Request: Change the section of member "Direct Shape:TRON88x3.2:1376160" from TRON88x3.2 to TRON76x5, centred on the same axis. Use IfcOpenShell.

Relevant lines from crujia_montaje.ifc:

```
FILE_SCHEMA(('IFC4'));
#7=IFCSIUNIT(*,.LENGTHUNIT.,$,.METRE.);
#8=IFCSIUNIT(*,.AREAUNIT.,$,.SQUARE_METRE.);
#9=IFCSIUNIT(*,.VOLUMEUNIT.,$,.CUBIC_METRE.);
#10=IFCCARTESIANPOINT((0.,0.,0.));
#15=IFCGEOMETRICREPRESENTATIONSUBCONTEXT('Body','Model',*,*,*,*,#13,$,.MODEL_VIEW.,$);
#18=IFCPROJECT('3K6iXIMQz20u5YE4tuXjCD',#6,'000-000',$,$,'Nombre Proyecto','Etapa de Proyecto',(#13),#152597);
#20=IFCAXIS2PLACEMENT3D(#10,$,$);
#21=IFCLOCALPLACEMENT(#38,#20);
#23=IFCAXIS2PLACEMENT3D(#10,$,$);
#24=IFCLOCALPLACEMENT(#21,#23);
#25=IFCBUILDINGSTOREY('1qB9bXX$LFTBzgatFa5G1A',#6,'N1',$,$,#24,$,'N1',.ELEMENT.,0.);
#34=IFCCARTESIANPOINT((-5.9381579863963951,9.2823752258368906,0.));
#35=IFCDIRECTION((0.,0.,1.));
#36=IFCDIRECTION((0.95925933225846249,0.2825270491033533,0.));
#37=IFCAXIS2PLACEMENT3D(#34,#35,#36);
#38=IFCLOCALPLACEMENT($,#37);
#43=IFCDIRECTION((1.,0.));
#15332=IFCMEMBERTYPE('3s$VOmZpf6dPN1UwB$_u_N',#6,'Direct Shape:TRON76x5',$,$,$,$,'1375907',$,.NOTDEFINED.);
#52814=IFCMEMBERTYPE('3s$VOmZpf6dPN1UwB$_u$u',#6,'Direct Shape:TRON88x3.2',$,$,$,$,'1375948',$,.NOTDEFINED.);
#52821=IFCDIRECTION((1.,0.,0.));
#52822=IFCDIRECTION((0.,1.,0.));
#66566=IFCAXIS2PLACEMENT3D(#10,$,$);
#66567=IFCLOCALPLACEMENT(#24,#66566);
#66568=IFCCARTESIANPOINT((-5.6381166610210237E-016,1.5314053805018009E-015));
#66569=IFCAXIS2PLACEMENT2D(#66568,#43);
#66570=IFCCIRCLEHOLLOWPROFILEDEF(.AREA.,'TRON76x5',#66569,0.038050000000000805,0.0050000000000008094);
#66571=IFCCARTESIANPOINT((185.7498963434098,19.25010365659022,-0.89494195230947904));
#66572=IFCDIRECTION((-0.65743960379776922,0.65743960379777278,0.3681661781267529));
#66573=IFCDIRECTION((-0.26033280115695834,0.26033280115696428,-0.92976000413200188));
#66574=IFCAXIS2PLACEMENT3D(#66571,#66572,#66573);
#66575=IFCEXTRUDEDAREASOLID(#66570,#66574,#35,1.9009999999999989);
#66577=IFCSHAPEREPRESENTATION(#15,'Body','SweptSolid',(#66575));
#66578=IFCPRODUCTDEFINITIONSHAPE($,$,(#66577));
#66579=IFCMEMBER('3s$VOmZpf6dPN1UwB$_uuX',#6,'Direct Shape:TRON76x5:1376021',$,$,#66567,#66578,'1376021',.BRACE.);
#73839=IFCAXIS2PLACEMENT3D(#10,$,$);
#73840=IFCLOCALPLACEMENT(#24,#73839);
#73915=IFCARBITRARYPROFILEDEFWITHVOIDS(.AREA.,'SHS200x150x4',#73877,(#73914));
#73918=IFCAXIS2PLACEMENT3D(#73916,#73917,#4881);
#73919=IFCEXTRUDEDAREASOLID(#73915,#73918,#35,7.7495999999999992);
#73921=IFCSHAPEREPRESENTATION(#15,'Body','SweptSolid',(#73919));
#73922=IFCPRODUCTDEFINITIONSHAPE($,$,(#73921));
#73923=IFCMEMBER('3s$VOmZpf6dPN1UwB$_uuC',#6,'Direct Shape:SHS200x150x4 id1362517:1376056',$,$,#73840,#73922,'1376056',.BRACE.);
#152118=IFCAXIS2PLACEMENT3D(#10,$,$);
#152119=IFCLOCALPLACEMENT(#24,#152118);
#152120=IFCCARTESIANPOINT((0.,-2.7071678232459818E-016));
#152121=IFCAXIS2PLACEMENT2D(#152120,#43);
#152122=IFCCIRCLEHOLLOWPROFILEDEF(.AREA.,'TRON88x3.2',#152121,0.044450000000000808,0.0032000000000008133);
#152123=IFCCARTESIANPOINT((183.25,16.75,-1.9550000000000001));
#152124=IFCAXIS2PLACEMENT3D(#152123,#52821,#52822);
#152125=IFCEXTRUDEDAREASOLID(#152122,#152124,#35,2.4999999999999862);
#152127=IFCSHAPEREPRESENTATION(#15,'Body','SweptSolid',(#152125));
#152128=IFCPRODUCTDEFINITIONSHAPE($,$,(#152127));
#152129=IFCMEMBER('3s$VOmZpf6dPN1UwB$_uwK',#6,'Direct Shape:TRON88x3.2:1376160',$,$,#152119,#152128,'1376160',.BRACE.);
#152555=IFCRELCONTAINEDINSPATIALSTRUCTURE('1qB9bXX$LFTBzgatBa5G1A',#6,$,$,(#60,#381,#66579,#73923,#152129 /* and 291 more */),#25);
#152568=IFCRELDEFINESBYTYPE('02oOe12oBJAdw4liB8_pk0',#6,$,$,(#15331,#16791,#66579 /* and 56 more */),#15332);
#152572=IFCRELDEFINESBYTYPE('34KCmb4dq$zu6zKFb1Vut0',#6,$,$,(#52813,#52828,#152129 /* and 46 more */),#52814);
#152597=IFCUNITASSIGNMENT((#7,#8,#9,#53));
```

```python
import ifcopenshell
import ifcopenshell.api.type
import ifcopenshell.util.element
import ifcopenshell.util.representation

model = ifcopenshell.open("crujia_montaje.ifc")

member = model.by_id(152129)
source = next(p for p in model.by_type("IfcCircleHollowProfileDef") if p.ProfileName == "TRON76x5")

body = ifcopenshell.util.representation.get_representation(member, "Model", "Body")
solid = body.Items[0]
old_profile = solid.SweptArea

# Copy the section's sizes but keep this member's own profile position.
profile = ifcopenshell.util.element.copy(model, source)
profile.Position = old_profile.Position
solid.SweptArea = profile
if not model.get_total_inverses(old_profile):
    ifcopenshell.util.element.remove_deep2(model, old_profile)

new_type = model.by_id(15332)
ifcopenshell.api.type.assign_type(
    model, related_objects=[member], relating_type=new_type, should_map_representations=False
)
member.Name = member.Name.replace("TRON88x3.2", "TRON76x5")

print(solid.SweptArea)

model.write("crujia_montaje_v2.ifc")
```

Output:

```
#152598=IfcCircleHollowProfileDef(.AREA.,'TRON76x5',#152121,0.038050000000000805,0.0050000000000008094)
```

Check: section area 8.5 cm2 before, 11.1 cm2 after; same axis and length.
